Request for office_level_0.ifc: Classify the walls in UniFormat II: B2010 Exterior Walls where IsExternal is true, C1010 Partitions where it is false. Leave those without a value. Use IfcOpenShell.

First a look at what the model holds.

```python
import ifcopenshell
import ifcopenshell.util.element

model = ifcopenshell.open("office_level_0.ifc")
print(model.schema)
print("classifications:", [c.Name for c in model.by_type("IfcClassification")])
values = [ifcopenshell.util.element.get_pset(e, "Pset_WallCommon", "IsExternal") for e in model.by_type("IfcWall")]
for value in (True, False, None):
    print("IsExternal", value, values.count(value))
```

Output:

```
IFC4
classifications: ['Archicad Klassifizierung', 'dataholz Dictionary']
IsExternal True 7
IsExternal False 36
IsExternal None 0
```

```python
import ifcopenshell
import ifcopenshell.api.classification
import ifcopenshell.util.element

model = ifcopenshell.open("office_level_0.ifc")

system = ifcopenshell.api.classification.add_classification(model, classification="UniFormat II")

walls = model.by_type("IfcWall")
external = {e: ifcopenshell.util.element.get_pset(e, "Pset_WallCommon", "IsExternal") for e in walls}
for flag, code, name in ((True, "B2010", "Exterior Walls"), (False, "C1010", "Partitions")):
    products = [e for e in walls if external[e] is flag]
    ifcopenshell.api.classification.add_reference(
        model, products=products, classification=system, identification=code, name=name
    )
    print(code, len(products))

model.write("office_level_0_v2.ifc")
```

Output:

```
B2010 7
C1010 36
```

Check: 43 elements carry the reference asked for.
